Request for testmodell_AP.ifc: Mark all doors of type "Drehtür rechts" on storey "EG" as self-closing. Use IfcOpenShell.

First a look at what the model holds.

```python
import ifcopenshell
import ifcopenshell.util.element

model = ifcopenshell.open("testmodell_AP.ifc")
print(model.schema)
storey = next(s for s in model.by_type("IfcBuildingStorey") if s.Name == "EG")
doors = [e for e in ifcopenshell.util.element.get_decomposition(storey) if e.is_a("IfcDoor")]
seen = {}
for e in doors:
    element_type = ifcopenshell.util.element.get_type(e)
    key = (element_type.Name if element_type != e and element_type else None, ifcopenshell.util.element.get_pset(e, "Pset_DoorCommon", "SelfClosing"))
    seen[key] = seen.get(key, 0) + 1
for (name, value), count in sorted(seen.items(), key=str):
    print(count, "x", name, "|", value)
```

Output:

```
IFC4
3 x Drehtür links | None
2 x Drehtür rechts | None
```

```python
import ifcopenshell
import ifcopenshell.api.pset
import ifcopenshell.util.element

model = ifcopenshell.open("testmodell_AP.ifc")

storey = next(s for s in model.by_type("IfcBuildingStorey") if s.Name == "EG")
doors = [e for e in ifcopenshell.util.element.get_decomposition(storey) if e.is_a("IfcDoor")]

count = 0
for e in doors:
    element_type = ifcopenshell.util.element.get_type(e)
    if element_type in (None, e) or element_type.Name != "Drehtür rechts":
        continue
    # add_pset returns the element's existing set when there is one.
    pset = ifcopenshell.api.pset.add_pset(model, product=e, name="Pset_DoorCommon")
    ifcopenshell.api.pset.edit_pset(model, pset=pset, properties={"SelfClosing": True})
    count += 1

print(count, "doors updated")

model.write("testmodell_AP_v2.ifc")
```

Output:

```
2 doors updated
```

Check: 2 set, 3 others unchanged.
